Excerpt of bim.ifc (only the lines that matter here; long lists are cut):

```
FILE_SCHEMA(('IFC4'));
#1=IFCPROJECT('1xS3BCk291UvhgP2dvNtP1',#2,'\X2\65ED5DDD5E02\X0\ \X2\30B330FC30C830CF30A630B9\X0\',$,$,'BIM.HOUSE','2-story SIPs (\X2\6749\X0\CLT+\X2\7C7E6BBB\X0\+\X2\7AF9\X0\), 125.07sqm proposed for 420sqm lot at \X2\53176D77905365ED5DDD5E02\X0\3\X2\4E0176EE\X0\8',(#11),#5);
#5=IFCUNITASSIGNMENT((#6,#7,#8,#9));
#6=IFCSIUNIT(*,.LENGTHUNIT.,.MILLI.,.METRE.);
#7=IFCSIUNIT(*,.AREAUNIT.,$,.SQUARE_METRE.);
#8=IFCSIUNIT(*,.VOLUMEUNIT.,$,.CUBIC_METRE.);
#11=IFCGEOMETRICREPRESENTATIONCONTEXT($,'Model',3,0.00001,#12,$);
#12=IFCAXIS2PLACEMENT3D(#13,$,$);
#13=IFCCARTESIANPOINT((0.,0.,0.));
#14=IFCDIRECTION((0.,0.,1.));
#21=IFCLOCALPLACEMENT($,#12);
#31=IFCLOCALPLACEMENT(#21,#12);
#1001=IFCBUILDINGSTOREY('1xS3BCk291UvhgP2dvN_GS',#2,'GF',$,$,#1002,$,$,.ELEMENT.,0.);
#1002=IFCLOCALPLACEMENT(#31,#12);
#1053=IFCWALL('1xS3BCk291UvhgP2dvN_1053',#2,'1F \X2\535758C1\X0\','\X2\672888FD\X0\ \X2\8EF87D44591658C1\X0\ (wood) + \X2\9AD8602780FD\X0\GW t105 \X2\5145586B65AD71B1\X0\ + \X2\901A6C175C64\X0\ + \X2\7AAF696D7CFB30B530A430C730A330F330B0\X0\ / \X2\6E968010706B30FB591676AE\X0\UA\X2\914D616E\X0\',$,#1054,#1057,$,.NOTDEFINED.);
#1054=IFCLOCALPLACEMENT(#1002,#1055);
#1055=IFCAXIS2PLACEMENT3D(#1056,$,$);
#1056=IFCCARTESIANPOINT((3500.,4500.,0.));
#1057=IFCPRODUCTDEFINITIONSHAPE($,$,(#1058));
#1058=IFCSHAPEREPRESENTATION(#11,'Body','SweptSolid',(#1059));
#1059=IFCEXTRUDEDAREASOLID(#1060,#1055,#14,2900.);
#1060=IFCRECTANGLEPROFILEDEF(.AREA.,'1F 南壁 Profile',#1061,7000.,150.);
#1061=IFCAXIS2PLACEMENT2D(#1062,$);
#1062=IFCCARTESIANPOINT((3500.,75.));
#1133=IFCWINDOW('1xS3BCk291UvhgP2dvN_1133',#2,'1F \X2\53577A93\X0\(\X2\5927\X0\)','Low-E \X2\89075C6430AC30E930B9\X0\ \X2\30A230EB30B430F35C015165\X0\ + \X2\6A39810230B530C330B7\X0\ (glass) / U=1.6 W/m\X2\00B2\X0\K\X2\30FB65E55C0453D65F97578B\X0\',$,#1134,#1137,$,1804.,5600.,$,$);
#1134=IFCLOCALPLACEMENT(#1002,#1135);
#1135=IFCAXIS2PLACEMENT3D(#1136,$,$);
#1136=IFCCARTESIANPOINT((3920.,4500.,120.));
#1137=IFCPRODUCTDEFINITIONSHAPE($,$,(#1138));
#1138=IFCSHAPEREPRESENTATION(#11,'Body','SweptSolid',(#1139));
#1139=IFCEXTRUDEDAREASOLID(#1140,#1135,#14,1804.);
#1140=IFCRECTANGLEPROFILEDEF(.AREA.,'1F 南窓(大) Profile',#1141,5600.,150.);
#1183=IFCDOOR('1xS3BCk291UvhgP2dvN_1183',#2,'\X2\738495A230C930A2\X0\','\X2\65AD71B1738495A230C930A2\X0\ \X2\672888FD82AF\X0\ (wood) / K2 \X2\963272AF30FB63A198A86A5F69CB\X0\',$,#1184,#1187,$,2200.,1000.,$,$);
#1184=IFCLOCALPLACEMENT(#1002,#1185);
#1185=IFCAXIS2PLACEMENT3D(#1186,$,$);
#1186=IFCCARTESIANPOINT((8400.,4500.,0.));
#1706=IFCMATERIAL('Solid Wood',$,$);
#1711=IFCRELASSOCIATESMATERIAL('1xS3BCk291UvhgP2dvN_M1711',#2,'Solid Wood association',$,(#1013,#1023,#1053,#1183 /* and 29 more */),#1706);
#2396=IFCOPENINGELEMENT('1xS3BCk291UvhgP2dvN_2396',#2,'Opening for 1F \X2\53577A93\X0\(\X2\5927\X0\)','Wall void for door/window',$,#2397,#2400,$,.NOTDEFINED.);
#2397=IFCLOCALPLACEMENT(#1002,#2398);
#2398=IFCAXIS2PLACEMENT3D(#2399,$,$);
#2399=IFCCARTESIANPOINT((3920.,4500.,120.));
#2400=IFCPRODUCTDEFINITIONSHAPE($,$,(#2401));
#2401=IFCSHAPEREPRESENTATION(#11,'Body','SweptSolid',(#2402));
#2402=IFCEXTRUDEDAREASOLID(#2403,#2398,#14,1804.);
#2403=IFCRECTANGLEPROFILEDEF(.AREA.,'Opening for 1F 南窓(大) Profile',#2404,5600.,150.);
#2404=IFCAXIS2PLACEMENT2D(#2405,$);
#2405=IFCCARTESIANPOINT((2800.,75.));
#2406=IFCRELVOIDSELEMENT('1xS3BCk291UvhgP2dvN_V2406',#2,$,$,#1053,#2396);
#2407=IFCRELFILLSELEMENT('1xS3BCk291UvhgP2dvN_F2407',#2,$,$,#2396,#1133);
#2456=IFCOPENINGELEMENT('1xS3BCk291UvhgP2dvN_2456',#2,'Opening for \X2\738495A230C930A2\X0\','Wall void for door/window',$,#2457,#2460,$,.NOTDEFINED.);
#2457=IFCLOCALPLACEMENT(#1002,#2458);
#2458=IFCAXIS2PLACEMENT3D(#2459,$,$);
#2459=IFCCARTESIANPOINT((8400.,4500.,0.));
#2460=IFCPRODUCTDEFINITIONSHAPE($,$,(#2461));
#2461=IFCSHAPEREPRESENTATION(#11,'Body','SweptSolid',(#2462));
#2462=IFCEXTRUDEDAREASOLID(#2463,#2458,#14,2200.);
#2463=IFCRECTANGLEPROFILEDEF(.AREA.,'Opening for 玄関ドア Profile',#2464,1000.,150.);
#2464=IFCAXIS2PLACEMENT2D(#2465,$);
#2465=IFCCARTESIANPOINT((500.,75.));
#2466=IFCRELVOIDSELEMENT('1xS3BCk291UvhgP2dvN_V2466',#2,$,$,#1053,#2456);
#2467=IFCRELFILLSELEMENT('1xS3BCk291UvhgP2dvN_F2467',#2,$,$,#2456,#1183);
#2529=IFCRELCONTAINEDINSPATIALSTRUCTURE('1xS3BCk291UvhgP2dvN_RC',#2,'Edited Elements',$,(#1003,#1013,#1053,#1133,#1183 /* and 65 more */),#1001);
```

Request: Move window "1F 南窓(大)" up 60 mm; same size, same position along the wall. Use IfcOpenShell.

```python
import numpy as np
import ifcopenshell
import ifcopenshell.api.geometry
import ifcopenshell.util.placement
import ifcopenshell.util.unit

model = ifcopenshell.open("bim.ifc")
unit_scale = ifcopenshell.util.unit.calculate_unit_scale(model)

window = model.by_id(1133)
opening = window.FillsVoids[0].RelatingOpeningElement
dz = 0.06 / unit_scale

shift = np.array([0.0, 0.0, dz])
# The window is not placed relative to its opening, so move both.
for product in (opening, window):
    matrix = ifcopenshell.util.placement.get_local_placement(product.ObjectPlacement)
    matrix[:3, 3] += shift
    ifcopenshell.api.geometry.edit_object_placement(model, product=product, matrix=matrix, is_si=False)

print(f"moved by {dz * unit_scale:+.3f} m")

model.write("bim_rev.ifc")
```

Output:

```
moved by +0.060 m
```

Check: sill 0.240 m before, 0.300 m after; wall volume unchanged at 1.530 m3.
